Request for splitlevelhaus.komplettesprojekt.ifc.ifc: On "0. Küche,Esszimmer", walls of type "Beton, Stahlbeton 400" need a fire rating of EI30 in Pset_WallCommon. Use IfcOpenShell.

First a look at what the model holds.

```python
import ifcopenshell
import ifcopenshell.util.element

model = ifcopenshell.open("splitlevelhaus.komplettesprojekt.ifc.ifc")
print(model.schema)
storey = next(s for s in model.by_type("IfcBuildingStorey") if s.Name == "0. Küche,Esszimmer")
walls = [e for e in ifcopenshell.util.element.get_decomposition(storey) if e.is_a("IfcWall")]
seen = {}
for e in walls:
    element_type = ifcopenshell.util.element.get_type(e)
    key = (element_type.Name if element_type != e and element_type else None, ifcopenshell.util.element.get_pset(e, "Pset_WallCommon", "FireRating"))
    seen[key] = seen.get(key, 0) + 1
for (name, value), count in sorted(seen.items(), key=str):
    print(count, "x", name, "|", value)
```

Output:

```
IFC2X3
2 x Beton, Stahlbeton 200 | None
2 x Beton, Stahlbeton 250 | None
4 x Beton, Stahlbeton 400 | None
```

```python
import ifcopenshell
import ifcopenshell.api.pset
import ifcopenshell.util.element

model = ifcopenshell.open("splitlevelhaus.komplettesprojekt.ifc.ifc")

storey = next(s for s in model.by_type("IfcBuildingStorey") if s.Name == "0. Küche,Esszimmer")
walls = [e for e in ifcopenshell.util.element.get_decomposition(storey) if e.is_a("IfcWall")]

count = 0
for e in walls:
    element_type = ifcopenshell.util.element.get_type(e)
    if element_type in (None, e) or element_type.Name != "Beton, Stahlbeton 400":
        continue
    # add_pset returns the element's existing set when there is one.
    pset = ifcopenshell.api.pset.add_pset(model, product=e, name="Pset_WallCommon")
    ifcopenshell.api.pset.edit_pset(model, pset=pset, properties={"FireRating": "EI30"})
    count += 1

print(count, "walls updated")

model.write("splitlevelhaus.komplettesprojekt.ifc-out.ifc")
```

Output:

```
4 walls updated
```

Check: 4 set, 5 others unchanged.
